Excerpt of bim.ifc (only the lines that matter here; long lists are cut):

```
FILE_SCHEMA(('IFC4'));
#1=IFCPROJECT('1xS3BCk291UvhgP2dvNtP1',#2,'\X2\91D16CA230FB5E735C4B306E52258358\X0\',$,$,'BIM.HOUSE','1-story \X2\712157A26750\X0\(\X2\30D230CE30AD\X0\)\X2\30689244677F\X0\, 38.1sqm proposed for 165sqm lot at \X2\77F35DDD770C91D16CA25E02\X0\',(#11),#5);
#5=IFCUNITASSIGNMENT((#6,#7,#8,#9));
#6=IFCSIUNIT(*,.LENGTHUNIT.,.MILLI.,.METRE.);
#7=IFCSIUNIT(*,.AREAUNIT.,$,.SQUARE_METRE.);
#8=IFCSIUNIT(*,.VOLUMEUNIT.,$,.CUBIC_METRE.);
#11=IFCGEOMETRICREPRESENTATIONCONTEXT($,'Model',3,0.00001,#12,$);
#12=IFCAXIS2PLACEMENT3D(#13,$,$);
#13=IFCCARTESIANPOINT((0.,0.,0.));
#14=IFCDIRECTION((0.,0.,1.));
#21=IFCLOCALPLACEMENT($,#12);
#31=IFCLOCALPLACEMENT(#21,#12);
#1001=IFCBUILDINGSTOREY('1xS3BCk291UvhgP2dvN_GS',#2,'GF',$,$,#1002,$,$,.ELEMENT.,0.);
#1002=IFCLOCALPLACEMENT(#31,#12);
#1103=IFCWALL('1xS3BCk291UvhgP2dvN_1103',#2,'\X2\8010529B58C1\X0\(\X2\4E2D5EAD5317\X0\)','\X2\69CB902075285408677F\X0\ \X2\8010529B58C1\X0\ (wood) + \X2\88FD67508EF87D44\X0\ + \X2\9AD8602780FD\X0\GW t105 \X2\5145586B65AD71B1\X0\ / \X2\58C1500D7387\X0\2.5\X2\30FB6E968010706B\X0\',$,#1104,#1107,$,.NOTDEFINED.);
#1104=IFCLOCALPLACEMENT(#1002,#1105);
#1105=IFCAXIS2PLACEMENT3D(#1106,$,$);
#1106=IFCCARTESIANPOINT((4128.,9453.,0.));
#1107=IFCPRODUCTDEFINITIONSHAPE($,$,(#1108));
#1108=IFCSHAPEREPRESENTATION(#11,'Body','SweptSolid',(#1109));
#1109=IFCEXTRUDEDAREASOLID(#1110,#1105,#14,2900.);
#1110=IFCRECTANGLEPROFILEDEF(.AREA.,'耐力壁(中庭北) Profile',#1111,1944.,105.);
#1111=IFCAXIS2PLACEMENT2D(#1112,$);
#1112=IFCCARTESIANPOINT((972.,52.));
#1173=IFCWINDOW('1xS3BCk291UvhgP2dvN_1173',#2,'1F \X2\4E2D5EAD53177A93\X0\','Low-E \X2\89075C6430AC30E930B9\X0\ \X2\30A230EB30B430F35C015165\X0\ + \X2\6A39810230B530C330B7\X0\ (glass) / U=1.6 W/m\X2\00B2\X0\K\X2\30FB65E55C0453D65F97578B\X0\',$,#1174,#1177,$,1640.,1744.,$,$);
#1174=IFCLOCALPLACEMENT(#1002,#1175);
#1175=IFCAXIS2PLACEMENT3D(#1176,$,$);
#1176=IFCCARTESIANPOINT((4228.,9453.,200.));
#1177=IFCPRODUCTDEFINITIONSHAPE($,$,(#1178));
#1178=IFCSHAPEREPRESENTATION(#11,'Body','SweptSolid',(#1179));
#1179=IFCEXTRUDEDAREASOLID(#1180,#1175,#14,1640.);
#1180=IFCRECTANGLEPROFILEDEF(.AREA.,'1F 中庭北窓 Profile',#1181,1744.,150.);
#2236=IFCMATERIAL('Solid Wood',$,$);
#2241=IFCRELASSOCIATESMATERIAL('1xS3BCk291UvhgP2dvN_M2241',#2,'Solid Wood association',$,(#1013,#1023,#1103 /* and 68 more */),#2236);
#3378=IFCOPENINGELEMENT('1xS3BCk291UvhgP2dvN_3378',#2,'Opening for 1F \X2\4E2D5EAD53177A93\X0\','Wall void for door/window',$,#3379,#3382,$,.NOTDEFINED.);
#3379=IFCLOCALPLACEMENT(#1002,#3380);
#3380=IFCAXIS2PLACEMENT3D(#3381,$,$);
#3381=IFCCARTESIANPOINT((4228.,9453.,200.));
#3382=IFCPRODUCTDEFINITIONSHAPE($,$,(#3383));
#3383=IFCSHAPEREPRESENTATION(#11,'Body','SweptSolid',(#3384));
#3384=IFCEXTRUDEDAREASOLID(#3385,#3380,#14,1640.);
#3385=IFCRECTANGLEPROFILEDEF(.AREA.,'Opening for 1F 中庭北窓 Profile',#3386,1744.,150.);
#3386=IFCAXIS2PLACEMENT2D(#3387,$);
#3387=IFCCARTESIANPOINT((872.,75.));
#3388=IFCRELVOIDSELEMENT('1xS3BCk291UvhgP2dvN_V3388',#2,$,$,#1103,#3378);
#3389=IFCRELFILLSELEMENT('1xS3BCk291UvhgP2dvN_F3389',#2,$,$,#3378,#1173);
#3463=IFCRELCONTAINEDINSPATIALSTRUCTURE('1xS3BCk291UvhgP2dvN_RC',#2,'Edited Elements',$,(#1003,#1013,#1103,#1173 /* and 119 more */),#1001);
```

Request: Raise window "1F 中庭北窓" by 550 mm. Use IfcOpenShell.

```python
import numpy as np
import ifcopenshell
import ifcopenshell.api.geometry
import ifcopenshell.util.placement
import ifcopenshell.util.unit

model = ifcopenshell.open("bim.ifc")
unit_scale = ifcopenshell.util.unit.calculate_unit_scale(model)

window = model.by_guid("1xS3BCk291UvhgP2dvN_1173")
opening = window.FillsVoids[0].RelatingOpeningElement
dz = 550.0

shift = np.array([0.0, 0.0, dz])
# The window is not placed relative to its opening, so move both.
for product in (opening, window):
    matrix = ifcopenshell.util.placement.get_local_placement(product.ObjectPlacement)
    matrix[:3, 3] += shift
    ifcopenshell.api.geometry.edit_object_placement(model, product=product, matrix=matrix, is_si=False)

print(f"moved by {dz * unit_scale:+.3f} m")

model.write("bim_updated.ifc")
```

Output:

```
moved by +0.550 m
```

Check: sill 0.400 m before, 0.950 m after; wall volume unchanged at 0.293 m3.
